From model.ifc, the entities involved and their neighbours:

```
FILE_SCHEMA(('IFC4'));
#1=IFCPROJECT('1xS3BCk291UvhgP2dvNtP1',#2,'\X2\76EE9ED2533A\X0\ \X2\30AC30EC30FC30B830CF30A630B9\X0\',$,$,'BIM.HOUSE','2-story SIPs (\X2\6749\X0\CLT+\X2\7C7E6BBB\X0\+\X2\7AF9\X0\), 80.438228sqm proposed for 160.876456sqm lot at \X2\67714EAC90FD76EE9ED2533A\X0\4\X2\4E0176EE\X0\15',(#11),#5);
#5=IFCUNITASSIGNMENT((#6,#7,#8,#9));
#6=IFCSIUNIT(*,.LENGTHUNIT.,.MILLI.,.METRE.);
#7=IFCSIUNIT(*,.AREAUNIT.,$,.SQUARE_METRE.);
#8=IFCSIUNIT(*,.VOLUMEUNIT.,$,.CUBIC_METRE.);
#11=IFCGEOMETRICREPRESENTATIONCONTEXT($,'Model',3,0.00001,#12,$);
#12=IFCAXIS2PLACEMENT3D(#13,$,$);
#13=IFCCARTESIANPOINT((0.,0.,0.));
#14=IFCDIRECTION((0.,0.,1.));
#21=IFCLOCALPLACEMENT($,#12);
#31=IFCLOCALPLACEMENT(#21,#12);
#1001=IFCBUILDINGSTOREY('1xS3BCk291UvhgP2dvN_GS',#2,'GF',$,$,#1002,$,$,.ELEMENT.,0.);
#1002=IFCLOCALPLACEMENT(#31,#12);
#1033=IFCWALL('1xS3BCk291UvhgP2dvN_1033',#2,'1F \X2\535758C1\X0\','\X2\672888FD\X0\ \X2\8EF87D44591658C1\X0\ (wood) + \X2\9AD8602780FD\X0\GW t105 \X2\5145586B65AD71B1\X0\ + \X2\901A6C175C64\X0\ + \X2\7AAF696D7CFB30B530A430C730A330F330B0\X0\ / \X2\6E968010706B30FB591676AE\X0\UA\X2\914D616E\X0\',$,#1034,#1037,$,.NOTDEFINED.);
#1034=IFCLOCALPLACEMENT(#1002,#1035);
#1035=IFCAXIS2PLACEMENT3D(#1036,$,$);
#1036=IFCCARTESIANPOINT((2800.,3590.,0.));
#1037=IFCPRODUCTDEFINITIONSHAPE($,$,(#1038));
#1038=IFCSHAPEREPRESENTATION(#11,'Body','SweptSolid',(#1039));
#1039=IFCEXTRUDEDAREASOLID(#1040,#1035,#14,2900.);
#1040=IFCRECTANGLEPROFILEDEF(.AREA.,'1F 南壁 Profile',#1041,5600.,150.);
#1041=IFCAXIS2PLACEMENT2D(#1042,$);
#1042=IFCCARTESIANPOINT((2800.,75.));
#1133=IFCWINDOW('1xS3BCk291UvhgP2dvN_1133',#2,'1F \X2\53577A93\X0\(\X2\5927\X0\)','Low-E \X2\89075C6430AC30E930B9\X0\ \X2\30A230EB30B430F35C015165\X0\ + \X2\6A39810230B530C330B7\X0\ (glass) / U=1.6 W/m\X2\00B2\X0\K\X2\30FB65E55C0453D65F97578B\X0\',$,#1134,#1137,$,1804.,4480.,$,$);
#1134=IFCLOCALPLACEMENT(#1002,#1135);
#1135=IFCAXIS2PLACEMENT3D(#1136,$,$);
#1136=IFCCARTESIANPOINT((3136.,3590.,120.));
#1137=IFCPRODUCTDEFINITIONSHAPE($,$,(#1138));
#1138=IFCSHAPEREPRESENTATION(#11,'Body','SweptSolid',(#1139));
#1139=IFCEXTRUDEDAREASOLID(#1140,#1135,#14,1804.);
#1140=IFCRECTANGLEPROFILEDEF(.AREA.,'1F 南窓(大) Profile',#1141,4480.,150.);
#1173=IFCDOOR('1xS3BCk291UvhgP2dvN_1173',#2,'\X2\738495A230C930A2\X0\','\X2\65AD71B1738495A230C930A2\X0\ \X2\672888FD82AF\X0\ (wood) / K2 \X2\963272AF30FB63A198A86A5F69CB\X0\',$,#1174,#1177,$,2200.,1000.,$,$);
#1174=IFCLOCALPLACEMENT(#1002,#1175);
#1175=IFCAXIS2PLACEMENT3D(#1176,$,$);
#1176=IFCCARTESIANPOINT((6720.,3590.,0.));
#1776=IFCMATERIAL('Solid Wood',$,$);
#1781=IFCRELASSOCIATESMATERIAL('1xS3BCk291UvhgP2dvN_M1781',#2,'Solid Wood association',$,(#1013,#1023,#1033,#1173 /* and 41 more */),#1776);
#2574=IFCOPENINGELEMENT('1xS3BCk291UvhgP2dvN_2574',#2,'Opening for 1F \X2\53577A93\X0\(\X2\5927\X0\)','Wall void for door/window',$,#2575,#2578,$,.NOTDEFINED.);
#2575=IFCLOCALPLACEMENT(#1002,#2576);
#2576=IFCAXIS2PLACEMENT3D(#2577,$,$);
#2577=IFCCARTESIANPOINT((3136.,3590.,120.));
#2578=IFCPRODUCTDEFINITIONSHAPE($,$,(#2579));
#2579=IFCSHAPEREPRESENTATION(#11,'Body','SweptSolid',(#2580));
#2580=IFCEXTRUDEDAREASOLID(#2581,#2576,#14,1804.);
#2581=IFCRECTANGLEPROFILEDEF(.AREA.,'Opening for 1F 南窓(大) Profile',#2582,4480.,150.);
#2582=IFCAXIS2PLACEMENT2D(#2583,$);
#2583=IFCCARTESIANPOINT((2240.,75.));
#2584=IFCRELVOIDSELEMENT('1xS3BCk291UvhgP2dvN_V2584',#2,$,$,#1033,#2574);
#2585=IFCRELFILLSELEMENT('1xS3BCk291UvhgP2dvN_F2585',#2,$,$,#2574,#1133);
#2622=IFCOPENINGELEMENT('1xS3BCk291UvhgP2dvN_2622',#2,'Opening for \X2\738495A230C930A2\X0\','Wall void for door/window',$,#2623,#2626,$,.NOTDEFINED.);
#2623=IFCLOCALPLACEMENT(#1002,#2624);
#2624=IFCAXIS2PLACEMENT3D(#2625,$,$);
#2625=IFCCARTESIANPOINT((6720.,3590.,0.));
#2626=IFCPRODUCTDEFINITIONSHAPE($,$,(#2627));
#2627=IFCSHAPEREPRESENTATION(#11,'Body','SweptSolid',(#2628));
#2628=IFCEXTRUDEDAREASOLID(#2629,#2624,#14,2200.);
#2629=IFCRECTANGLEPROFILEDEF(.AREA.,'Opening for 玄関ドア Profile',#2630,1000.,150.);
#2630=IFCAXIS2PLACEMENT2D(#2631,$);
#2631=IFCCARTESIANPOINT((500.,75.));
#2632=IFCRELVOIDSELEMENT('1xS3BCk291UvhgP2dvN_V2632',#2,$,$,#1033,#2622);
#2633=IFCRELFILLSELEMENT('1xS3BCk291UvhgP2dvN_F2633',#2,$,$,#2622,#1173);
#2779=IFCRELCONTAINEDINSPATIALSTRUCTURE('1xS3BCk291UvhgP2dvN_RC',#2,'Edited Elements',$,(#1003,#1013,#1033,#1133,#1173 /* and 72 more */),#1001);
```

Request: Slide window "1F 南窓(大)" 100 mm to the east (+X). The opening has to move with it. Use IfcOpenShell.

```python
import ifcopenshell
import ifcopenshell.api.geometry
import ifcopenshell.util.placement
import ifcopenshell.util.unit

model = ifcopenshell.open("model.ifc")
unit_scale = ifcopenshell.util.unit.calculate_unit_scale(model)

window = model.by_guid("1xS3BCk291UvhgP2dvN_1133")
opening = window.FillsVoids[0].RelatingOpeningElement
wall = opening.VoidsElements[0].RelatingBuildingElement

wall_matrix = ifcopenshell.util.placement.get_local_placement(wall.ObjectPlacement)
shift = wall_matrix[:3, 0] * 0.1 / unit_scale
before = ifcopenshell.util.placement.get_local_placement(window.ObjectPlacement)[:3, 3].copy()

# The window is not placed relative to its opening, so move both.
for product in (opening, window):
    matrix = ifcopenshell.util.placement.get_local_placement(product.ObjectPlacement)
    matrix[:3, 3] += shift
    ifcopenshell.api.geometry.edit_object_placement(model, product=product, matrix=matrix, is_si=False)

after = ifcopenshell.util.placement.get_local_placement(window.ObjectPlacement)[:3, 3]
print("window moved by", (after - before).round(3) + 0.0)

model.write("model_updated.ifc")
```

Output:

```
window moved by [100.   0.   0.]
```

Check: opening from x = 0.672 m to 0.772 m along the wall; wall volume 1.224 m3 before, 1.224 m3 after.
